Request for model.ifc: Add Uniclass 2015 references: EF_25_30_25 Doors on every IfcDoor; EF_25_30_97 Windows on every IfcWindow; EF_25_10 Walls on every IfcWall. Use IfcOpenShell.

First a look at what the model holds.

```python
import ifcopenshell

model = ifcopenshell.open("model.ifc")
print(model.schema)
print("classifications:", [c.Name for c in model.by_type("IfcClassification")])
for ifc_class in ("IfcDoor", "IfcRoof", "IfcStair", "IfcWall", "IfcWindow"):
    print(ifc_class, len(model.by_type(ifc_class)))
```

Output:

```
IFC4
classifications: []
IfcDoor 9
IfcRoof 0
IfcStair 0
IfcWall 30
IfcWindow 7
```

```python
import ifcopenshell
import ifcopenshell.api.classification

model = ifcopenshell.open("model.ifc")

system = ifcopenshell.api.classification.add_classification(model, classification="Uniclass 2015")

codes = {
    "IfcDoor": ("EF_25_30_25", "Doors"),
    "IfcWindow": ("EF_25_30_97", "Windows"),
    "IfcWall": ("EF_25_10", "Walls"),
}
for ifc_class, (code, name) in codes.items():
    products = model.by_type(ifc_class)
    ifcopenshell.api.classification.add_reference(
        model, products=products, classification=system, identification=code, name=name
    )
    print(code, len(products))

model.write("model-out.ifc")
```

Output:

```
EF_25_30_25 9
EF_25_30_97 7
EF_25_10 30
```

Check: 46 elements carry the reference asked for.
